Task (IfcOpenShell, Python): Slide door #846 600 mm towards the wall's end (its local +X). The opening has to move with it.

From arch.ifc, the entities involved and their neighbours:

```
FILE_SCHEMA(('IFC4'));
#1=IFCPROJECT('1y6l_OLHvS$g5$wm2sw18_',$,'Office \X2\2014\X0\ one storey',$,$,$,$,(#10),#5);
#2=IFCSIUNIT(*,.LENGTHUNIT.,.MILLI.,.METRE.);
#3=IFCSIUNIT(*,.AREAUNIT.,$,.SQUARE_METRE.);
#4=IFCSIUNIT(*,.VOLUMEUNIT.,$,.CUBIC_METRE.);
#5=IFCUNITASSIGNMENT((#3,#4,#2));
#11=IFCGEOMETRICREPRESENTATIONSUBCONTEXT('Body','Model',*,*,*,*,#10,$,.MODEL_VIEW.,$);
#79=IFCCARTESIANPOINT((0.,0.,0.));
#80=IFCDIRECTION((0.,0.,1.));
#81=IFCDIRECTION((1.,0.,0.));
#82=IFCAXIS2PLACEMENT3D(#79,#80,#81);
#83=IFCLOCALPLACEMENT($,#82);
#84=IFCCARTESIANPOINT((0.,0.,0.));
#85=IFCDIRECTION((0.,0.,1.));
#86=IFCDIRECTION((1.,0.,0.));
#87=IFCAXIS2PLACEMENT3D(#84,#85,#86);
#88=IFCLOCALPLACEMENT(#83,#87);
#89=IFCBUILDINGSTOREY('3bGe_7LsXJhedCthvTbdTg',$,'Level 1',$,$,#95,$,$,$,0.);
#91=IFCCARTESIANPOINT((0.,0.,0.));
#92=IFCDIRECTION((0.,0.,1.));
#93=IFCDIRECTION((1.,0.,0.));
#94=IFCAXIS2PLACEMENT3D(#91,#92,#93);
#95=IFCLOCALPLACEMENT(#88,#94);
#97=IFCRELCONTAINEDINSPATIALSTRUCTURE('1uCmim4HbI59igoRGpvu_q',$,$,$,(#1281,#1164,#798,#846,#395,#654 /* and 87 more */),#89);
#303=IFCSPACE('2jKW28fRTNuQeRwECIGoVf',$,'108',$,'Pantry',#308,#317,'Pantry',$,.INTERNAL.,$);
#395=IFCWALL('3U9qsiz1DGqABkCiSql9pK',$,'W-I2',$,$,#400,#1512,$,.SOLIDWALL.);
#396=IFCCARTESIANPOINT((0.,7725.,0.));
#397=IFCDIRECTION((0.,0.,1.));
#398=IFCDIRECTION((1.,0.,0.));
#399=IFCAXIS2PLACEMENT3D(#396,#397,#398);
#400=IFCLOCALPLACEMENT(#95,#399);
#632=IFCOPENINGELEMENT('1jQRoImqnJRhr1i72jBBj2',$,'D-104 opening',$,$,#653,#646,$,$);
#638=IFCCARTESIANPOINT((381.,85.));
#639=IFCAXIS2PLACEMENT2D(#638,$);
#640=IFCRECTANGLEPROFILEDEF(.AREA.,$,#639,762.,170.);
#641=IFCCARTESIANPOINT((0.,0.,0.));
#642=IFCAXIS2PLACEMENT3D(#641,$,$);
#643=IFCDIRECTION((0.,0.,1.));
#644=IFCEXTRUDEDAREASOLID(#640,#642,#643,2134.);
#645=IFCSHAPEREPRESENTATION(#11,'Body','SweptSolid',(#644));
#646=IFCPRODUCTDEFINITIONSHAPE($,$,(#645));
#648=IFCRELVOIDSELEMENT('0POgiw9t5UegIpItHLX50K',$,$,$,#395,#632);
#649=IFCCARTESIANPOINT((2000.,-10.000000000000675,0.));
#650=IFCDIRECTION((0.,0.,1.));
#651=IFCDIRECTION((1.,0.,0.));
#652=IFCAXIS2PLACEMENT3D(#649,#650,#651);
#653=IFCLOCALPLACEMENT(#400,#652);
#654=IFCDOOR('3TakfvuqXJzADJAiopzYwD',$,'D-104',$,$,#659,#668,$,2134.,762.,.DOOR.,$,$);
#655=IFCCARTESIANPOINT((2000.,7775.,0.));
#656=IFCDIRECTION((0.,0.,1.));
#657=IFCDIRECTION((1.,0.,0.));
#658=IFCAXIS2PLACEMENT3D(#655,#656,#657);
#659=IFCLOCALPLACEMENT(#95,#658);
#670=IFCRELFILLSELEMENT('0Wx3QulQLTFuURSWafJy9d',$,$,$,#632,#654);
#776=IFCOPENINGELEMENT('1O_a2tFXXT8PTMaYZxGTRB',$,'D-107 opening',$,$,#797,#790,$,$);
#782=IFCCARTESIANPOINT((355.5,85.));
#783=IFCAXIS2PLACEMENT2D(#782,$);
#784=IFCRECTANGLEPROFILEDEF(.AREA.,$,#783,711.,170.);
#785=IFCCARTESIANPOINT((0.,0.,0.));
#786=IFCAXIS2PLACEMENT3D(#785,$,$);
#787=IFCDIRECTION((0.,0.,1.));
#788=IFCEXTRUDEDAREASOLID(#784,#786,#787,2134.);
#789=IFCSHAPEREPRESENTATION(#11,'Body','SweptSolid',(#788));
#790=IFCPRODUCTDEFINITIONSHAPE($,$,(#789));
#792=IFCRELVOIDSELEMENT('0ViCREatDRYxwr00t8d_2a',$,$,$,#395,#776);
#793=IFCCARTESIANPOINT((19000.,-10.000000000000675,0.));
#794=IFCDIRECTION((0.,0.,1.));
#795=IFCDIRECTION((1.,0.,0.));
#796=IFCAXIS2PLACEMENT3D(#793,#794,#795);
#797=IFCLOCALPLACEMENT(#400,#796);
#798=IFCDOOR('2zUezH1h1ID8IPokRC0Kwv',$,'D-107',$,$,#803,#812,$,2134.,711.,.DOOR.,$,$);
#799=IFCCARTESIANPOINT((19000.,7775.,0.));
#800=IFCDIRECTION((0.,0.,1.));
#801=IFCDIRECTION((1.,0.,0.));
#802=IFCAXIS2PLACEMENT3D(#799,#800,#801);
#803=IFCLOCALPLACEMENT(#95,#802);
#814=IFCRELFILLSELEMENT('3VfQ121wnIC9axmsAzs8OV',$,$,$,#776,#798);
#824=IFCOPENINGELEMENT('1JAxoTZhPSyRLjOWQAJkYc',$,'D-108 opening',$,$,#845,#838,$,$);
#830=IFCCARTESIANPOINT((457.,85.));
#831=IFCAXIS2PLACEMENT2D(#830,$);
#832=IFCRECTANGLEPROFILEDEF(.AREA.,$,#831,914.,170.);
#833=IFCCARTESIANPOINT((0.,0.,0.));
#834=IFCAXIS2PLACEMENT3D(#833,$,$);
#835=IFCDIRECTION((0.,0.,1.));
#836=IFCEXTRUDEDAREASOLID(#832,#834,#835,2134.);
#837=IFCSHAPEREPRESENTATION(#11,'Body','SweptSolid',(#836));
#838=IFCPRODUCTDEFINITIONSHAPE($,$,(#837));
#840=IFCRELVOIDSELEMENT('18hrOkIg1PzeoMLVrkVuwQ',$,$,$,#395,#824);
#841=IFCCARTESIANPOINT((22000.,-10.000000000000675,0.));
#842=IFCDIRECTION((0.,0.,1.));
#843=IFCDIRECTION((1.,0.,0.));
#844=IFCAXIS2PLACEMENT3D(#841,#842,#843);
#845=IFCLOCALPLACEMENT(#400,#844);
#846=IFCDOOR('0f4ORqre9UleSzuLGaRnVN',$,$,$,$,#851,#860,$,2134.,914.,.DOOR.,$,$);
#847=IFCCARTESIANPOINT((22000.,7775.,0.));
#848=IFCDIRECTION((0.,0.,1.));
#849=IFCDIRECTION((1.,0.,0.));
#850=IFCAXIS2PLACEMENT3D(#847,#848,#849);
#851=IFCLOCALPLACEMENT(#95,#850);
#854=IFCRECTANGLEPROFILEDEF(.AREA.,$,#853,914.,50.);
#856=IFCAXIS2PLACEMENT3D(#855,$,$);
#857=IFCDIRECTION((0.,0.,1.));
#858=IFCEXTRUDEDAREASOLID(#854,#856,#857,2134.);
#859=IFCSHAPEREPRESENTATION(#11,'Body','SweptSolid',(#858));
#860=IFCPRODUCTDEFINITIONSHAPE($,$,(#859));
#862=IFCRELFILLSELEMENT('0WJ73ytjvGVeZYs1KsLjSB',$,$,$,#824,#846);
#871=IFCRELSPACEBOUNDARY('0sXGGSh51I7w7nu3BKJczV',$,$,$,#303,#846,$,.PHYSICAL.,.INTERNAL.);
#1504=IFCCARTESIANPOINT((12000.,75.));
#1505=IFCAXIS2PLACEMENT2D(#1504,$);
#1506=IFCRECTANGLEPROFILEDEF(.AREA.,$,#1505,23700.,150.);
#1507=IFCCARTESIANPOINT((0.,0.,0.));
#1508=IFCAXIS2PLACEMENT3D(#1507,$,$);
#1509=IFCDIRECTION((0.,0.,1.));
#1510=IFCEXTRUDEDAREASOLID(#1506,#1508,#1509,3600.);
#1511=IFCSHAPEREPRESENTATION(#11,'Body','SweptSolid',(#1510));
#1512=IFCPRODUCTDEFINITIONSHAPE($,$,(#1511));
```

```python
import ifcopenshell
import ifcopenshell.api.geometry
import ifcopenshell.util.placement
import ifcopenshell.util.unit

model = ifcopenshell.open("arch.ifc")
unit_scale = ifcopenshell.util.unit.calculate_unit_scale(model)

door = model.by_id(846)
opening = door.FillsVoids[0].RelatingOpeningElement
wall = opening.VoidsElements[0].RelatingBuildingElement

wall_matrix = ifcopenshell.util.placement.get_local_placement(wall.ObjectPlacement)
shift = wall_matrix[:3, 0] * 0.6 / unit_scale
before = ifcopenshell.util.placement.get_local_placement(door.ObjectPlacement)[:3, 3].copy()

# The door is not placed relative to its opening, so move both.
for product in (opening, door):
    matrix = ifcopenshell.util.placement.get_local_placement(product.ObjectPlacement)
    matrix[:3, 3] += shift
    ifcopenshell.api.geometry.edit_object_placement(model, product=product, matrix=matrix, is_si=False)

after = ifcopenshell.util.placement.get_local_placement(door.ObjectPlacement)[:3, 3]
print("door moved by", (after - before).round(3) + 0.0)

model.write("arch-out.ifc")
```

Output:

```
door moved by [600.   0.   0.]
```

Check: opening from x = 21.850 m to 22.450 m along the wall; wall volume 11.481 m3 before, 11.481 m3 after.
